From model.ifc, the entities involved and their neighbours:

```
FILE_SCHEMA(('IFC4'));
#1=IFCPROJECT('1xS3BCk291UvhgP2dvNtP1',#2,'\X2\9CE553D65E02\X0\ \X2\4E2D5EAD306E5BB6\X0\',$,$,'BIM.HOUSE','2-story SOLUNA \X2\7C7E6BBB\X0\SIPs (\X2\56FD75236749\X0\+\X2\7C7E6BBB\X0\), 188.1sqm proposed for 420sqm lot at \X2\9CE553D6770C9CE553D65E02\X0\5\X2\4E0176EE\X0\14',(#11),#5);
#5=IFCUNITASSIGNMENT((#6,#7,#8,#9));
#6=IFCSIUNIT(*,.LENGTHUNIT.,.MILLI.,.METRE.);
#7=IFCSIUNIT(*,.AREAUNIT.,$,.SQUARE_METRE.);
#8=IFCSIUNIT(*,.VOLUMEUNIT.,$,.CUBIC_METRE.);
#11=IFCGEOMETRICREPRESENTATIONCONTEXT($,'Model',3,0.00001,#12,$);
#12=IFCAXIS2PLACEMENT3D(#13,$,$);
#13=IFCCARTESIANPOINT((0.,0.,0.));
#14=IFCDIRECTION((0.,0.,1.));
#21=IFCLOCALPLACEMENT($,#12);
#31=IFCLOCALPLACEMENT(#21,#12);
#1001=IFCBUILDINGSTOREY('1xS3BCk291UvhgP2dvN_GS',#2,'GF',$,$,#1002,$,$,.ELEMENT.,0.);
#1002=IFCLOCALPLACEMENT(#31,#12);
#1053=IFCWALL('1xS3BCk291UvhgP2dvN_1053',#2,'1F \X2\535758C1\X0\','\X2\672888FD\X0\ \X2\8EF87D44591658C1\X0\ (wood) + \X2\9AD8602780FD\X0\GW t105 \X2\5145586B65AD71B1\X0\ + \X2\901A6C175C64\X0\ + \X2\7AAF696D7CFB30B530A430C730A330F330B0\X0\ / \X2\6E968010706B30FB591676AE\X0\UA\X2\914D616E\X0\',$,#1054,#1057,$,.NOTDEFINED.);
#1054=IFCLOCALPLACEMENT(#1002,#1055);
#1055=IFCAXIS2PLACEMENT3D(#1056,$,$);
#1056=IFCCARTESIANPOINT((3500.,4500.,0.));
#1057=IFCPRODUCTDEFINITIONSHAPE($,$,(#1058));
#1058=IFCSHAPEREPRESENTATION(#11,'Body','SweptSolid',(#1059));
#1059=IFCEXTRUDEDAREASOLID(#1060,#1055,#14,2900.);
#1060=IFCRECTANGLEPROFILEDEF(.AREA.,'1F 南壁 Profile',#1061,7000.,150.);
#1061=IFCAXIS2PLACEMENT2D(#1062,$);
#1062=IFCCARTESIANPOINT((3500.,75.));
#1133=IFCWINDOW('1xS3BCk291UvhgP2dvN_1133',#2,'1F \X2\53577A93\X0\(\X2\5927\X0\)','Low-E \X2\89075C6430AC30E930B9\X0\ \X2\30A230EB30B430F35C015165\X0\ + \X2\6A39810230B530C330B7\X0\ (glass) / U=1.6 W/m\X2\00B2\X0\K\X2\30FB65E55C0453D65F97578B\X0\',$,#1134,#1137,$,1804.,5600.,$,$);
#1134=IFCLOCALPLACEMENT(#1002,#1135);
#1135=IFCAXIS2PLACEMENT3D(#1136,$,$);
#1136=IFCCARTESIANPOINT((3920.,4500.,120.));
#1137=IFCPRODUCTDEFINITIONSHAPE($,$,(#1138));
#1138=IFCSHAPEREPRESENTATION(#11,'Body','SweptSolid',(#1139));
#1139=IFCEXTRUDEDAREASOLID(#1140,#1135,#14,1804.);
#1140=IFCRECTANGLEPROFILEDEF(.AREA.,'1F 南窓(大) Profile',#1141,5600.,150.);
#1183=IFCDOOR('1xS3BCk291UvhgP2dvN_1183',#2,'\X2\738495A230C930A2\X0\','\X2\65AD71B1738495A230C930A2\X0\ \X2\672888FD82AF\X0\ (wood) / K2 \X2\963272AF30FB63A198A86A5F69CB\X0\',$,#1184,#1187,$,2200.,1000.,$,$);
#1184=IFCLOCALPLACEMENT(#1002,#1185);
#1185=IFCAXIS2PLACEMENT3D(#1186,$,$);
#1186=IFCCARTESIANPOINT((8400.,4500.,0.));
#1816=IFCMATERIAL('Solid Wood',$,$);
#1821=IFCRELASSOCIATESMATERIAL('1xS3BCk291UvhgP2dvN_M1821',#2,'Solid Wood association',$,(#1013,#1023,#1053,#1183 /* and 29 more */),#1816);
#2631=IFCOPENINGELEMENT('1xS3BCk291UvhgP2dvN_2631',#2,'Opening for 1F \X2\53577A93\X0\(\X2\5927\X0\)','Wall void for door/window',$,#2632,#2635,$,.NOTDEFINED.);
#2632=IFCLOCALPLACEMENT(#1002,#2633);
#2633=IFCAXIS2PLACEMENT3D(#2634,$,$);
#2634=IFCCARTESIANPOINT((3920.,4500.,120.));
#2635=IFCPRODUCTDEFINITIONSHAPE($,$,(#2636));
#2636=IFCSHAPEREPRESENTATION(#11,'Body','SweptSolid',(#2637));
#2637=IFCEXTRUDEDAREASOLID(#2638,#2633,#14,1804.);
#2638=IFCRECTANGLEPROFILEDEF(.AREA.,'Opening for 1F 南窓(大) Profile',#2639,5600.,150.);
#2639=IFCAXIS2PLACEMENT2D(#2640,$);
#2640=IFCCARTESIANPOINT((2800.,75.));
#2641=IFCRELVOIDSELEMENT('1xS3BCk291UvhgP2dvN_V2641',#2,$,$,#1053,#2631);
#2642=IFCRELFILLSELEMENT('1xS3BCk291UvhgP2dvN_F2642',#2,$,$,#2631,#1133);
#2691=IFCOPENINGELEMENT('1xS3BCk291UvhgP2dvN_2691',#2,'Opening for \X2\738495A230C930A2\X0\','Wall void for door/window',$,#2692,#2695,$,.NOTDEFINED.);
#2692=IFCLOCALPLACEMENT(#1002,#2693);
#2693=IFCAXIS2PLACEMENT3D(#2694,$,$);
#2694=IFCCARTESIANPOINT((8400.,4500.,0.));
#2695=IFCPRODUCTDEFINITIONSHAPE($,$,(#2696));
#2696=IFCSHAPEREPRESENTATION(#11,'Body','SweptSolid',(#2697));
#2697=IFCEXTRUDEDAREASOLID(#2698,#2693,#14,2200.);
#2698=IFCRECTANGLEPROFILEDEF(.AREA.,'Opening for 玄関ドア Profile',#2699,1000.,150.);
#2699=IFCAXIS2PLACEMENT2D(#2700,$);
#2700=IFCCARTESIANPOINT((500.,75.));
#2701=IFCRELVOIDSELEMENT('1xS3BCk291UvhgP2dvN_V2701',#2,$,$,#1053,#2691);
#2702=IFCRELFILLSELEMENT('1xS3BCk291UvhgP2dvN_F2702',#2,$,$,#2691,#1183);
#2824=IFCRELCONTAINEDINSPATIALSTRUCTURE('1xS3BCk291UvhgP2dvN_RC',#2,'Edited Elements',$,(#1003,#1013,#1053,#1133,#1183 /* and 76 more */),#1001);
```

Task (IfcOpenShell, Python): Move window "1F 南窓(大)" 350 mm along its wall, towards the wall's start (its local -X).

```python
import ifcopenshell
import ifcopenshell.api.geometry
import ifcopenshell.util.placement

model = ifcopenshell.open("model.ifc")

window = model.by_guid("1xS3BCk291UvhgP2dvN_1133")
opening = window.FillsVoids[0].RelatingOpeningElement
wall = opening.VoidsElements[0].RelatingBuildingElement

wall_matrix = ifcopenshell.util.placement.get_local_placement(wall.ObjectPlacement)
shift = wall_matrix[:3, 0] * -350.0
before = ifcopenshell.util.placement.get_local_placement(window.ObjectPlacement)[:3, 3].copy()

# The window is not placed relative to its opening, so move both.
for product in (opening, window):
    matrix = ifcopenshell.util.placement.get_local_placement(product.ObjectPlacement)
    matrix[:3, 3] += shift
    ifcopenshell.api.geometry.edit_object_placement(model, product=product, matrix=matrix, is_si=False)

after = ifcopenshell.util.placement.get_local_placement(window.ObjectPlacement)[:3, 3]
print("window moved by", (after - before).round(3) + 0.0)

model.write("model-out.ifc")
```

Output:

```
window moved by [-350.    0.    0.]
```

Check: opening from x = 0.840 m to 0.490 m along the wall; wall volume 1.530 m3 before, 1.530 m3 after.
